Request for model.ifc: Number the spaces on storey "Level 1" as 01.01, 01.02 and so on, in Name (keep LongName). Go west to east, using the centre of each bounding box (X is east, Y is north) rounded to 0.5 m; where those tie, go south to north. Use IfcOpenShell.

First a look at what the model holds.

```python
import ifcopenshell
import ifcopenshell.util.element
import ifcopenshell.util.placement

model = ifcopenshell.open("model.ifc")
print(model.schema)
storey = next(s for s in model.by_type("IfcBuildingStorey") if s.Name == "Level 1")
spaces = [e for e in ifcopenshell.util.element.get_decomposition(storey) if e.is_a("IfcSpace")]
for e in sorted(spaces, key=lambda e: e.id()):
    origin = ifcopenshell.util.placement.get_local_placement(e.ObjectPlacement)[:3, 3]
    print(e.id(), e.Name, e.LongName, origin.round(2) + 0.0, sep=" | ")
```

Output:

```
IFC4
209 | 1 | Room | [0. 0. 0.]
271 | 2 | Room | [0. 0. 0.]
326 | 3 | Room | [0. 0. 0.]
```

```python
import ifcopenshell
import ifcopenshell.geom
import ifcopenshell.util.element
import ifcopenshell.util.shape

model = ifcopenshell.open("model.ifc")
settings = ifcopenshell.geom.settings()
settings.set("use-world-coords", True)


def centre(element):
    shape = ifcopenshell.geom.create_shape(settings, element)
    return ifcopenshell.util.shape.get_bbox_centroid(shape.geometry)


storey = next(s for s in model.by_type("IfcBuildingStorey") if s.Name == "Level 1")
spaces = [e for e in ifcopenshell.util.element.get_decomposition(storey) if e.is_a("IfcSpace")]

# Insertion points can sit at a corner or the storey origin, so sort by the geometry (in metres).
centres = {e: centre(e) for e in spaces}
spaces.sort(key=lambda e: (round(centres[e][0] / 0.5), centres[e][1]))

for i, e in enumerate(spaces, start=1):
    number = f"01.{i:02d}"
    e.Name = number
    print(e.id(), number)

model.write("model_rev.ifc")
```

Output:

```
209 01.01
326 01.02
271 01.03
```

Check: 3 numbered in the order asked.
